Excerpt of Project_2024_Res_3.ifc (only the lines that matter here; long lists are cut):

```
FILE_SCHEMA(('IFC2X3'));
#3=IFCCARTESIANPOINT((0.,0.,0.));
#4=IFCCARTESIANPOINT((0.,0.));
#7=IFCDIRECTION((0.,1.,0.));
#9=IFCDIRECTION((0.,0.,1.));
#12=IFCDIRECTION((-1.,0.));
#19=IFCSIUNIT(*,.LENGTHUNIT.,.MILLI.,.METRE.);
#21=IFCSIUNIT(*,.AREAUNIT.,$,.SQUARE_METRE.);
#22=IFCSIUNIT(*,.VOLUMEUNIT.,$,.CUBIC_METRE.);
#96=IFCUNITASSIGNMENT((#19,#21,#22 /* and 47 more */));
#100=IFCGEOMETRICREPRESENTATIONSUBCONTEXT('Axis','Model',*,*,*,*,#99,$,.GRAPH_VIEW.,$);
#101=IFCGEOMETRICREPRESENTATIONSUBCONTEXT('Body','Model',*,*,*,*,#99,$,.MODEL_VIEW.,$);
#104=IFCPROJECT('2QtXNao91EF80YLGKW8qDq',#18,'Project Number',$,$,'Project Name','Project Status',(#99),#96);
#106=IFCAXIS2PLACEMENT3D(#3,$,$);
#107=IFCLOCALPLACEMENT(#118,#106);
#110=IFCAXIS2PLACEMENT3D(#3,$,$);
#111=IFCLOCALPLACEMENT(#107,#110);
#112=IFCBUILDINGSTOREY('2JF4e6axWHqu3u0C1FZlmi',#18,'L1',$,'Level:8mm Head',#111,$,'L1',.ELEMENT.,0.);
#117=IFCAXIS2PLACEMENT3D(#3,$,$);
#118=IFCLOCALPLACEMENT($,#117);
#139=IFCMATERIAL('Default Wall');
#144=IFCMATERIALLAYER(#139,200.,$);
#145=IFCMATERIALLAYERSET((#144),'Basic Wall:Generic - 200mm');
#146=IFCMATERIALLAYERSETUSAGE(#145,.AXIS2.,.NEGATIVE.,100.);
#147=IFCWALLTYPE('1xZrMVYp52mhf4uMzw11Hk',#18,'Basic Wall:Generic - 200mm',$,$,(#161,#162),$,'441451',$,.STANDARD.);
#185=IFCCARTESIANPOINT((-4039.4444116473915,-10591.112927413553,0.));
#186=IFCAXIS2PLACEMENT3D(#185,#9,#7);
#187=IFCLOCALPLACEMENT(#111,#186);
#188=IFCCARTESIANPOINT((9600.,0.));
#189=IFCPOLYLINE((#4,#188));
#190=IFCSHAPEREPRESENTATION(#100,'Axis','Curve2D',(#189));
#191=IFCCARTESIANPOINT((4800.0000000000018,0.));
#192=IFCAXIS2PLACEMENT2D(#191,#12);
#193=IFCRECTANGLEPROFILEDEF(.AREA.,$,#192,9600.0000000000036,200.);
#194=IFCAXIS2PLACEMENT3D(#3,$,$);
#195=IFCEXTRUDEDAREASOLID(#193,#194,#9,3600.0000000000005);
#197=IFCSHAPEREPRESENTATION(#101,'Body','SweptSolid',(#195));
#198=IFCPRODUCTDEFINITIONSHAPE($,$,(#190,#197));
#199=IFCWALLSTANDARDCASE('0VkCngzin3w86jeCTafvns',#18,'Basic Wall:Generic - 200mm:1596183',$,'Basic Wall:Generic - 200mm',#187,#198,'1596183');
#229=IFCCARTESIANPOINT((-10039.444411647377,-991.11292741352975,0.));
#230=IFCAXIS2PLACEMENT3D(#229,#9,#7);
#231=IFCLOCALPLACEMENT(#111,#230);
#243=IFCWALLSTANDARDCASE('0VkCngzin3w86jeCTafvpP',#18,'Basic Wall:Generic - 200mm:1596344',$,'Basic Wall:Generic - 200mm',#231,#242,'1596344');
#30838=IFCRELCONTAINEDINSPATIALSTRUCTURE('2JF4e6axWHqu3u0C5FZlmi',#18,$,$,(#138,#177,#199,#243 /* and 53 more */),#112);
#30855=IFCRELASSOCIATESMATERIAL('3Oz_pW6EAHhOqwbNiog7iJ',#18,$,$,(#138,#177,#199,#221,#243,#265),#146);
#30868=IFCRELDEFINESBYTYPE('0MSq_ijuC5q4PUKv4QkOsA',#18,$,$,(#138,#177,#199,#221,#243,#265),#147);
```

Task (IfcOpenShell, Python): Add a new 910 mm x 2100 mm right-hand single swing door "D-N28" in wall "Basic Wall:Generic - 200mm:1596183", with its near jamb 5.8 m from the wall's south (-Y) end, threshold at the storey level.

```python
import numpy as np
import ifcopenshell
import ifcopenshell.api.feature
import ifcopenshell.api.geometry
import ifcopenshell.api.root
import ifcopenshell.api.spatial
import ifcopenshell.api.type
import ifcopenshell.geom
import ifcopenshell.util.element
import ifcopenshell.util.placement
import ifcopenshell.util.representation
import ifcopenshell.util.shape
import ifcopenshell.util.unit

model = ifcopenshell.open("Project_2024_Res_3.ifc")
unit_scale = ifcopenshell.util.unit.calculate_unit_scale(model)
settings = ifcopenshell.geom.settings()


def volume(element):
    """Net volume in cubic metres, openings subtracted."""
    shape = ifcopenshell.geom.create_shape(settings, element)
    return ifcopenshell.util.shape.get_volume(shape.geometry)


wall = model.by_guid("0VkCngzin3w86jeCTafvns")
storey = ifcopenshell.util.element.get_container(wall, ifc_class="IfcBuildingStorey")
context = ifcopenshell.util.representation.get_context(model, "Model", "Body", "MODEL_VIEW")
before = volume(wall)

width, height, from_end, sill = 0.91, 2.1, 5.8, 0.0  # metres

# The wall runs along its own X axis, and the end named is its -X end.
wall_shape = ifcopenshell.geom.create_shape(settings, wall)
x, y, z = ifcopenshell.util.shape.get_vertices(wall_shape.geometry).T
start = x.min() + from_end
face, thickness = float(y.min()), float(y.max() - y.min())
wall_matrix = ifcopenshell.util.placement.get_local_placement(wall.ObjectPlacement)
level = ifcopenshell.util.placement.get_local_placement(storey.ObjectPlacement)[2, 3]


def in_wall(x, y):
    """Placement at x, y metres in the wall's axes, at sill height."""
    matrix = wall_matrix.copy()
    matrix[:, 3] = wall_matrix @ np.array([x / unit_scale, y / unit_scale, 0.0, 1.0])
    matrix[2, 3] = level + sill / unit_scale
    return matrix


# Opening: a box that overshoots both wall faces by 50 mm.
opening = ifcopenshell.api.root.create_entity(model, ifc_class="IfcOpeningElement")
box = ifcopenshell.api.geometry.add_wall_representation(
    model, context=context, length=width, height=height, thickness=thickness + 0.1
)
ifcopenshell.api.geometry.assign_representation(model, product=opening, representation=box)
ifcopenshell.api.geometry.edit_object_placement(model, product=opening, matrix=in_wall(start, face - 0.05), is_si=False)
ifcopenshell.api.feature.add_feature(model, feature=opening, element=wall)

door = ifcopenshell.api.root.create_entity(model, ifc_class="IfcDoor", name="D-N28")
door.OverallWidth, door.OverallHeight = width / unit_scale, height / unit_scale
body = ifcopenshell.api.geometry.add_door_representation(
    model,
    context=context,
    overall_width=door.OverallWidth,
    overall_height=door.OverallHeight,
    operation_type="SINGLE_SWING_RIGHT",
    lining_properties={"LiningDepth": thickness / unit_scale, "ThresholdDepth": thickness / unit_scale},
)
ifcopenshell.api.geometry.assign_representation(model, product=door, representation=body)
ifcopenshell.api.spatial.assign_container(model, products=[door], relating_structure=storey)
fills = ifcopenshell.api.feature.add_filling(model, opening=opening, element=door)
fills.OwnerHistory = door.OwnerHistory  # required in IFC2X3

# IFC2X3 keeps the operation on the door style.
style = ifcopenshell.api.root.create_entity(model, ifc_class="IfcDoorStyle", name="D-N28")
style.OperationType, style.ConstructionType = "SINGLE_SWING_RIGHT", "NOTDEFINED"
style.ParameterTakesPrecedence = style.Sizeable = False
ifcopenshell.api.type.assign_type(model, related_objects=[door], relating_type=style)

# The lining spans the wall, so the door starts at the wall face.
ifcopenshell.api.geometry.edit_object_placement(model, product=door, matrix=in_wall(start, face), is_si=False)

after = volume(wall)

print(f"wall volume {before:.3f} -> {after:.3f} m3")

model.write("Project_2024_Res_3-out.ifc")
```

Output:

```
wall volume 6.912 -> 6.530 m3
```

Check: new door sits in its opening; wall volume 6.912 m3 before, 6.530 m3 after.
